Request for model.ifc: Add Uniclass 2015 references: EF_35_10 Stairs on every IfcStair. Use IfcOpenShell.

First a look at what the model holds.

```python
import ifcopenshell

model = ifcopenshell.open("model.ifc")
print(model.schema)
print("classifications:", [c.Name for c in model.by_type("IfcClassification")])
for ifc_class in ("IfcDoor", "IfcRoof", "IfcStair", "IfcWall", "IfcWindow"):
    print(ifc_class, len(model.by_type(ifc_class)))
```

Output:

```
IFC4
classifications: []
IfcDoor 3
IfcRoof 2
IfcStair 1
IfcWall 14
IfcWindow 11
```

```python
import ifcopenshell
import ifcopenshell.api.classification

model = ifcopenshell.open("model.ifc")

system = ifcopenshell.api.classification.add_classification(model, classification="Uniclass 2015")

codes = {
    "IfcStair": ("EF_35_10", "Stairs"),
}
for ifc_class, (code, name) in codes.items():
    products = model.by_type(ifc_class)
    ifcopenshell.api.classification.add_reference(
        model, products=products, classification=system, identification=code, name=name
    )
    print(code, len(products))

model.write("model_v2.ifc")
```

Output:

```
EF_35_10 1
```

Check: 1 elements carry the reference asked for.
